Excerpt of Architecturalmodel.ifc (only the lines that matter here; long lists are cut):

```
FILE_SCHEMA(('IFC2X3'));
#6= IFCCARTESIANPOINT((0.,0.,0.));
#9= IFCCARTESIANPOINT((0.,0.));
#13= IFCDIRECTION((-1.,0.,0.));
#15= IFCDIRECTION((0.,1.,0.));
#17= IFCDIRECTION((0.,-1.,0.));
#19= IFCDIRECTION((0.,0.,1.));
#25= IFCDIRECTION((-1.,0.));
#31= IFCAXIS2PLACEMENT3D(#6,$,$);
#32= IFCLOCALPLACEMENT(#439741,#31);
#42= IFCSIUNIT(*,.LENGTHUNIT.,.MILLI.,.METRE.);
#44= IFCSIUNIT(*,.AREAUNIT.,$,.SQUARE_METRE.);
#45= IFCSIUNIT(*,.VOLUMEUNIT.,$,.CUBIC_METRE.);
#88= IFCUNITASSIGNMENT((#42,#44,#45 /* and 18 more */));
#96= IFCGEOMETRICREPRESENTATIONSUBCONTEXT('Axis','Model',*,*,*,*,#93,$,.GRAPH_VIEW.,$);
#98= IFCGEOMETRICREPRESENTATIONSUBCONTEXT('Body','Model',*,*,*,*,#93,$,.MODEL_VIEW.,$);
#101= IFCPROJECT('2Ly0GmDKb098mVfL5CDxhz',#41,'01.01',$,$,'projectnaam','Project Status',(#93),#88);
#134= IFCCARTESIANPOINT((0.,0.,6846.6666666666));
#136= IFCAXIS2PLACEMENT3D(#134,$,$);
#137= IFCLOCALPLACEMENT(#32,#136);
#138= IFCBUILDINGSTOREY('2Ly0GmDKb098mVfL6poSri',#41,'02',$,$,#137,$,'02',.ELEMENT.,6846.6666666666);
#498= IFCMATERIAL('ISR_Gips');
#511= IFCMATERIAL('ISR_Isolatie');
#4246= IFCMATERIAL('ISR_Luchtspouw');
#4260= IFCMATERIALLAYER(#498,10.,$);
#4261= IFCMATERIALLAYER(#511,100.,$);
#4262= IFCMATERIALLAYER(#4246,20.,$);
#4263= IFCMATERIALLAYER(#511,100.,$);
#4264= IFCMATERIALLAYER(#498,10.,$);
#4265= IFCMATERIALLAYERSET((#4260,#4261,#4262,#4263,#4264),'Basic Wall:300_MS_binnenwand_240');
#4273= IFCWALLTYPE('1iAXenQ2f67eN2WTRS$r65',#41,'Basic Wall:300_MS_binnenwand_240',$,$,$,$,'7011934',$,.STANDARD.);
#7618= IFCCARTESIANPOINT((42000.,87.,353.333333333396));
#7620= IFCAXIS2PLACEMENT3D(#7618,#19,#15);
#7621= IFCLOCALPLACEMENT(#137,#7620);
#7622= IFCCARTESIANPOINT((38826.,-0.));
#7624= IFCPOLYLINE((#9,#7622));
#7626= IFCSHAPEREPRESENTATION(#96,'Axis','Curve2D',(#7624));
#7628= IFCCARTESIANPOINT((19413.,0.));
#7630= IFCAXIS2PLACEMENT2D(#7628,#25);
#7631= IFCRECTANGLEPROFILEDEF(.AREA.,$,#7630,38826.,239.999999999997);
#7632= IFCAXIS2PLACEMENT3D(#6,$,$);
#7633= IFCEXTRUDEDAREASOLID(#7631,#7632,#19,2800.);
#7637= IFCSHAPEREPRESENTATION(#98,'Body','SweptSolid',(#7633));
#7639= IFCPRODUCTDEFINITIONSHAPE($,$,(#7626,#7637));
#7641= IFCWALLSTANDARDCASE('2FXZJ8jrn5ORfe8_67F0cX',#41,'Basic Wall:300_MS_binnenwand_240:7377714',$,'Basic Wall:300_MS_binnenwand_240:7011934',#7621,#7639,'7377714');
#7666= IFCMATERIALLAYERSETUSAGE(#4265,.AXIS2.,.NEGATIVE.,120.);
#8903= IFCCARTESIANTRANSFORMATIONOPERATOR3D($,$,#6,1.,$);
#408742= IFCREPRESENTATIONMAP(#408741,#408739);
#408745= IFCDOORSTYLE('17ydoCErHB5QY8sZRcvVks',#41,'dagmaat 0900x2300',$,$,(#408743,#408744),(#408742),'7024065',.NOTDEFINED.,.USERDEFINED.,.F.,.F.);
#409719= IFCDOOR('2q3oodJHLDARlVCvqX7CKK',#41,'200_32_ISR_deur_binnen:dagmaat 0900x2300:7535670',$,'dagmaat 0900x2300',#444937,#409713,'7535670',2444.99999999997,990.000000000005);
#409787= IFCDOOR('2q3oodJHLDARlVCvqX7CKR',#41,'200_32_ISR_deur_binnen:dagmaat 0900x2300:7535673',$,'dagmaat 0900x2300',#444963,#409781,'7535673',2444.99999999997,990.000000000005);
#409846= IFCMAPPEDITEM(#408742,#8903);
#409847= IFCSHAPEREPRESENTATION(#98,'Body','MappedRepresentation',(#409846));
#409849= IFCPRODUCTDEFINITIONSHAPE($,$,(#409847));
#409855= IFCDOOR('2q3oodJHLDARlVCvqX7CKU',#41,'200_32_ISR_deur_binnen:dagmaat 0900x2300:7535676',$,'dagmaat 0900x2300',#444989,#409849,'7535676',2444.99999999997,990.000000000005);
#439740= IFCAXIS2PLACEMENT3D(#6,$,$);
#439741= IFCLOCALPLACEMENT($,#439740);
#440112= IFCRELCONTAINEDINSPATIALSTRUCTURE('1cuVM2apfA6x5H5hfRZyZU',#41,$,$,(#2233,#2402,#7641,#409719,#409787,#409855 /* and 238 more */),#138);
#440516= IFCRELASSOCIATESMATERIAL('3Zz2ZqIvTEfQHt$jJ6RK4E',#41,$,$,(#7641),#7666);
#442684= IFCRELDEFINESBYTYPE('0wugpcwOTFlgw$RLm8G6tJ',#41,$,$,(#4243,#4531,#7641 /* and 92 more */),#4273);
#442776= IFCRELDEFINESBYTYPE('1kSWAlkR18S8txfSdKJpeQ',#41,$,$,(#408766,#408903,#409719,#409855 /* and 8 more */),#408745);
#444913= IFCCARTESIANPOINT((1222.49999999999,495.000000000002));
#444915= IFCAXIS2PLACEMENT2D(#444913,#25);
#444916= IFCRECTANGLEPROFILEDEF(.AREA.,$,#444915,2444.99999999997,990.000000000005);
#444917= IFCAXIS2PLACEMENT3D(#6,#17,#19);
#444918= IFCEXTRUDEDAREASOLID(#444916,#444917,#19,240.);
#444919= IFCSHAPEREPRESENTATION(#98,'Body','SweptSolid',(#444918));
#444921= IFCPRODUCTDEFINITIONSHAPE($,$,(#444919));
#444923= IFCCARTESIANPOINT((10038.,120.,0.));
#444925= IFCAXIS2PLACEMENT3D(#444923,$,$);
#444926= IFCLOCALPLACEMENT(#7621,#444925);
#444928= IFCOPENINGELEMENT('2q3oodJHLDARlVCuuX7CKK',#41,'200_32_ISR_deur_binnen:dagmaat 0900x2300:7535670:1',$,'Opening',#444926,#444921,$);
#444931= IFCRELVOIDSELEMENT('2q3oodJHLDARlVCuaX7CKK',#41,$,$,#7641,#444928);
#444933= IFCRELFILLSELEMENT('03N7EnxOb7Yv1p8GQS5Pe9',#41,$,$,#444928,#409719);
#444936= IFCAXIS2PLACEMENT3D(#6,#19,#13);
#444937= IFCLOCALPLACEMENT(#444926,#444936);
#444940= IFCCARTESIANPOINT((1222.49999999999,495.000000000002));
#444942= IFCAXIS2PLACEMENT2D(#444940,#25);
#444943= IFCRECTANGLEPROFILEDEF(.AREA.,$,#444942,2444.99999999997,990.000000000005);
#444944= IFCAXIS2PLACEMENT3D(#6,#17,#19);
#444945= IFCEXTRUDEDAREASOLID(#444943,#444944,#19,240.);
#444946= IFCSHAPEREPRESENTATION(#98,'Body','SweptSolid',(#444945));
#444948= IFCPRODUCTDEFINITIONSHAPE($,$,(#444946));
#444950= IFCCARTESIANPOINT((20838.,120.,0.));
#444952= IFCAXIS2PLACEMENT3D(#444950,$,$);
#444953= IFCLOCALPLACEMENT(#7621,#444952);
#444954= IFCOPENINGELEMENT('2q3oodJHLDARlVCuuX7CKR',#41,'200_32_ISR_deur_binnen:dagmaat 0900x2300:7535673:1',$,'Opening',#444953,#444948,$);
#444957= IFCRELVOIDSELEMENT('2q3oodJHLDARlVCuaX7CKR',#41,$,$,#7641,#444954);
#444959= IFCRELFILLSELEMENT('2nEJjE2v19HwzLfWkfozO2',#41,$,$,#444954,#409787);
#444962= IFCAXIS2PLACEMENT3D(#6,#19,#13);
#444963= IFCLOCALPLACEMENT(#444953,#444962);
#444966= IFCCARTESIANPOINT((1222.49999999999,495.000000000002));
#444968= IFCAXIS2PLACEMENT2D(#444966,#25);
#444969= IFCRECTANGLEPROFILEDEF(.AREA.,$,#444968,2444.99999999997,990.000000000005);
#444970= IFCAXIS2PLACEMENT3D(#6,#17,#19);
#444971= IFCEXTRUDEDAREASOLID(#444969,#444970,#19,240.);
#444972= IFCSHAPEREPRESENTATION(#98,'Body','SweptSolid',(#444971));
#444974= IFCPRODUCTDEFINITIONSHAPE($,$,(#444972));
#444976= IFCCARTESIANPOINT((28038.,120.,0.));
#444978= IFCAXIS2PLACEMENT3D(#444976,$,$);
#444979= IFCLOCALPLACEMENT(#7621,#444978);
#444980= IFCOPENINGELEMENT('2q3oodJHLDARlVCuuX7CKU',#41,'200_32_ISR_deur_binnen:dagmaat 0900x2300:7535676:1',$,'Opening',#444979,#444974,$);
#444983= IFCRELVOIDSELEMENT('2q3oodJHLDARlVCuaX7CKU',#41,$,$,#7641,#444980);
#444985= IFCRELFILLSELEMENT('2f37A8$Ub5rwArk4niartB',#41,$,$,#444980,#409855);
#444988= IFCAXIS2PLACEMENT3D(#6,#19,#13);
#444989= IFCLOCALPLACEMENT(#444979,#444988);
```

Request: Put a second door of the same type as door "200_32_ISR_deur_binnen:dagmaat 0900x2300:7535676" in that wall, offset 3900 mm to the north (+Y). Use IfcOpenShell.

```python
import ifcopenshell
import ifcopenshell.api.feature
import ifcopenshell.api.geometry
import ifcopenshell.api.root
import ifcopenshell.geom
import ifcopenshell.util.element
import ifcopenshell.util.placement
import ifcopenshell.util.shape

model = ifcopenshell.open("Architecturalmodel.ifc")
settings = ifcopenshell.geom.settings()


def volume(element):
    """Net volume in cubic metres, openings subtracted."""
    shape = ifcopenshell.geom.create_shape(settings, element)
    return ifcopenshell.util.shape.get_volume(shape.geometry)


def reuse_history(source, copy):
    """copy_class also copies each property set's owner history, people and application; keep the originals."""
    for rel in copy.IsDefinedBy:
        if rel.is_a("IfcRelDefinesByProperties") and (history := rel.RelatingPropertyDefinition.OwnerHistory):
            rel.RelatingPropertyDefinition.OwnerHistory = source.OwnerHistory
            ifcopenshell.util.element.remove_deep2(model, history)


door = model.by_guid("2q3oodJHLDARlVCvqX7CKU")
opening = door.FillsVoids[0].RelatingOpeningElement
wall = opening.VoidsElements[0].RelatingBuildingElement
before = volume(wall)
shift = ifcopenshell.util.placement.get_local_placement(wall.ObjectPlacement)[:3, 0] * 3900.0

# copy_class copies the void relationship, type, container and properties, but no geometry.
new_opening = ifcopenshell.api.root.copy_class(model, product=opening)
new_opening.Representation = ifcopenshell.util.element.copy_deep(
    model, opening.Representation, exclude=["IfcGeometricRepresentationContext", "IfcRepresentationMap"]
)
new_opening.Name = "200_32_ISR_deur_binnen:dagmaat 0900x2300"
new_door = ifcopenshell.api.root.copy_class(model, product=door)
new_door.Representation = ifcopenshell.util.element.copy_deep(
    model, door.Representation, exclude=["IfcGeometricRepresentationContext", "IfcRepresentationMap"]
)
new_door.Name = "200_32_ISR_deur_binnen:dagmaat 0900x2300"
new_door.Tag = None
reuse_history(door, new_door)
fills = ifcopenshell.api.feature.add_filling(model, opening=new_opening, element=new_door)
fills.OwnerHistory = new_door.OwnerHistory  # required in IFC2X3

for old, new in ((opening, new_opening), (door, new_door)):
    matrix = ifcopenshell.util.placement.get_local_placement(old.ObjectPlacement)
    matrix[:3, 3] += shift
    ifcopenshell.api.geometry.edit_object_placement(model, product=new, matrix=matrix, is_si=False)

after = volume(wall)

print(f"wall volume {before:.3f} -> {after:.3f} m3")

model.write("Architecturalmodel_rev.ifc")
```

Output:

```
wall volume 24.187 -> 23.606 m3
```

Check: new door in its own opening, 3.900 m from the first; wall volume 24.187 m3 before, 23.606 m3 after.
